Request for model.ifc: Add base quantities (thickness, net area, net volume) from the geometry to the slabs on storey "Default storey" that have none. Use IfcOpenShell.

First a look at what the model holds.

```python
import ifcopenshell
import ifcopenshell.util.element
import ifcopenshell.util.unit

model = ifcopenshell.open("model.ifc")
print(model.schema)
for unit_type in ("LENGTHUNIT", "AREAUNIT", "VOLUMEUNIT"):
    print(unit_type, ifcopenshell.util.unit.calculate_unit_scale(model, unit_type))
storey = next(s for s in model.by_type("IfcBuildingStorey") if s.Name == "Default storey")
slabs = [e for e in ifcopenshell.util.element.get_decomposition(storey) if e.is_a("IfcSlab")]
for e in sorted(slabs, key=lambda e: e.id()):
    print(e.id(), e.is_a(), e.Name, list(ifcopenshell.util.element.get_psets(e, qtos_only=True)), sep=" | ")
```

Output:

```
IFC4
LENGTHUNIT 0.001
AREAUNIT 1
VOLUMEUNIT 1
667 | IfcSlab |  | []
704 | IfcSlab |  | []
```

```python
import ifcopenshell
import ifcopenshell.api.pset
import ifcopenshell.geom
import ifcopenshell.util.element
import ifcopenshell.util.shape
import ifcopenshell.util.unit

model = ifcopenshell.open("model.ifc")
unit_scale = ifcopenshell.util.unit.calculate_unit_scale(model)
area_scale = ifcopenshell.util.unit.calculate_unit_scale(model, "AREAUNIT")
volume_scale = ifcopenshell.util.unit.calculate_unit_scale(model, "VOLUMEUNIT")
settings = ifcopenshell.geom.settings()

storey = next(s for s in model.by_type("IfcBuildingStorey") if s.Name == "Default storey")
slabs = [e for e in ifcopenshell.util.element.get_decomposition(storey) if e.is_a("IfcSlab")]

for e in sorted(slabs, key=lambda e: e.id()):
    if ifcopenshell.util.element.get_psets(e, qtos_only=True, should_inherit=False):
        continue
    # Geometry comes back in metres, in the element's own axes.
    shape = ifcopenshell.geom.create_shape(settings, e)
    values = {
        "Width": ifcopenshell.util.shape.get_z(shape.geometry) / unit_scale,
        "NetArea": ifcopenshell.util.shape.get_footprint_area(shape.geometry) / area_scale,
        "NetVolume": ifcopenshell.util.shape.get_volume(shape.geometry) / volume_scale,
    }
    qto = ifcopenshell.api.pset.add_qto(model, product=e, name="Qto_SlabBaseQuantities")
    ifcopenshell.api.pset.edit_qto(model, qto=qto, properties=values)
    print(e.id(), {k: round(v, 3) for k, v in values.items()})

model.write("model-out.ifc")
```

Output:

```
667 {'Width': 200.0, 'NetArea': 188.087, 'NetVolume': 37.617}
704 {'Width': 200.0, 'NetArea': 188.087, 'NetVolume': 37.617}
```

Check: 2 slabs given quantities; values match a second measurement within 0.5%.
